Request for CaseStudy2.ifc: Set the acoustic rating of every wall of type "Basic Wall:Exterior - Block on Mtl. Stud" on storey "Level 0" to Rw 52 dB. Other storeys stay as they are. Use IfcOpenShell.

First a look at what the model holds.

```python
import ifcopenshell
import ifcopenshell.util.element

model = ifcopenshell.open("CaseStudy2.ifc")
print(model.schema)
storey = next(s for s in model.by_type("IfcBuildingStorey") if s.Name == "Level 0")
walls = [e for e in ifcopenshell.util.element.get_decomposition(storey) if e.is_a("IfcWall")]
seen = {}
for e in walls:
    element_type = ifcopenshell.util.element.get_type(e)
    key = (element_type.Name if element_type != e and element_type else None, ifcopenshell.util.element.get_pset(e, "Pset_WallCommon", "AcousticRating"))
    seen[key] = seen.get(key, 0) + 1
for (name, value), count in sorted(seen.items(), key=str):
    print(count, "x", name, "|", value)
```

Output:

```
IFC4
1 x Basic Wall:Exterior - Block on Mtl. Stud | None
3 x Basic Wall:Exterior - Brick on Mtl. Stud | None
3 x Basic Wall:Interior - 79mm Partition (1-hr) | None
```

```python
import ifcopenshell
import ifcopenshell.api.pset
import ifcopenshell.util.element

model = ifcopenshell.open("CaseStudy2.ifc")

storey = next(s for s in model.by_type("IfcBuildingStorey") if s.Name == "Level 0")
walls = [e for e in ifcopenshell.util.element.get_decomposition(storey) if e.is_a("IfcWall")]

count = 0
for e in walls:
    element_type = ifcopenshell.util.element.get_type(e)
    if element_type in (None, e) or element_type.Name != "Basic Wall:Exterior - Block on Mtl. Stud":
        continue
    # add_pset returns the element's existing set when there is one.
    pset = ifcopenshell.api.pset.add_pset(model, product=e, name="Pset_WallCommon")
    ifcopenshell.api.pset.edit_pset(model, pset=pset, properties={"AcousticRating": "Rw 52 dB"})
    count += 1

print(count, "walls updated")

model.write("CaseStudy2_v2.ifc")
```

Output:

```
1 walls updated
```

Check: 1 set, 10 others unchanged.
